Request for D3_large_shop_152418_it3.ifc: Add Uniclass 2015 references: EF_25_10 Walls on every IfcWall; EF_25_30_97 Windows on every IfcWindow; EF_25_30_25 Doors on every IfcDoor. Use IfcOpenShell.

First a look at what the model holds.

```python
import ifcopenshell

model = ifcopenshell.open("D3_large_shop_152418_it3.ifc")
print(model.schema)
print("classifications:", [c.Name for c in model.by_type("IfcClassification")])
for ifc_class in ("IfcDoor", "IfcRoof", "IfcStair", "IfcWall", "IfcWindow"):
    print(ifc_class, len(model.by_type(ifc_class)))
```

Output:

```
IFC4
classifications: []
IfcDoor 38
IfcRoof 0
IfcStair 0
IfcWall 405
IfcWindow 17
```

```python
import ifcopenshell
import ifcopenshell.api.classification

model = ifcopenshell.open("D3_large_shop_152418_it3.ifc")

system = ifcopenshell.api.classification.add_classification(model, classification="Uniclass 2015")

codes = {
    "IfcWall": ("EF_25_10", "Walls"),
    "IfcWindow": ("EF_25_30_97", "Windows"),
    "IfcDoor": ("EF_25_30_25", "Doors"),
}
for ifc_class, (code, name) in codes.items():
    products = model.by_type(ifc_class)
    ifcopenshell.api.classification.add_reference(
        model, products=products, classification=system, identification=code, name=name
    )
    print(code, len(products))

model.write("D3_large_shop_152418_it3_updated.ifc")
```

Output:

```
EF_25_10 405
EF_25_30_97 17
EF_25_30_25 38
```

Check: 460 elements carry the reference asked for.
